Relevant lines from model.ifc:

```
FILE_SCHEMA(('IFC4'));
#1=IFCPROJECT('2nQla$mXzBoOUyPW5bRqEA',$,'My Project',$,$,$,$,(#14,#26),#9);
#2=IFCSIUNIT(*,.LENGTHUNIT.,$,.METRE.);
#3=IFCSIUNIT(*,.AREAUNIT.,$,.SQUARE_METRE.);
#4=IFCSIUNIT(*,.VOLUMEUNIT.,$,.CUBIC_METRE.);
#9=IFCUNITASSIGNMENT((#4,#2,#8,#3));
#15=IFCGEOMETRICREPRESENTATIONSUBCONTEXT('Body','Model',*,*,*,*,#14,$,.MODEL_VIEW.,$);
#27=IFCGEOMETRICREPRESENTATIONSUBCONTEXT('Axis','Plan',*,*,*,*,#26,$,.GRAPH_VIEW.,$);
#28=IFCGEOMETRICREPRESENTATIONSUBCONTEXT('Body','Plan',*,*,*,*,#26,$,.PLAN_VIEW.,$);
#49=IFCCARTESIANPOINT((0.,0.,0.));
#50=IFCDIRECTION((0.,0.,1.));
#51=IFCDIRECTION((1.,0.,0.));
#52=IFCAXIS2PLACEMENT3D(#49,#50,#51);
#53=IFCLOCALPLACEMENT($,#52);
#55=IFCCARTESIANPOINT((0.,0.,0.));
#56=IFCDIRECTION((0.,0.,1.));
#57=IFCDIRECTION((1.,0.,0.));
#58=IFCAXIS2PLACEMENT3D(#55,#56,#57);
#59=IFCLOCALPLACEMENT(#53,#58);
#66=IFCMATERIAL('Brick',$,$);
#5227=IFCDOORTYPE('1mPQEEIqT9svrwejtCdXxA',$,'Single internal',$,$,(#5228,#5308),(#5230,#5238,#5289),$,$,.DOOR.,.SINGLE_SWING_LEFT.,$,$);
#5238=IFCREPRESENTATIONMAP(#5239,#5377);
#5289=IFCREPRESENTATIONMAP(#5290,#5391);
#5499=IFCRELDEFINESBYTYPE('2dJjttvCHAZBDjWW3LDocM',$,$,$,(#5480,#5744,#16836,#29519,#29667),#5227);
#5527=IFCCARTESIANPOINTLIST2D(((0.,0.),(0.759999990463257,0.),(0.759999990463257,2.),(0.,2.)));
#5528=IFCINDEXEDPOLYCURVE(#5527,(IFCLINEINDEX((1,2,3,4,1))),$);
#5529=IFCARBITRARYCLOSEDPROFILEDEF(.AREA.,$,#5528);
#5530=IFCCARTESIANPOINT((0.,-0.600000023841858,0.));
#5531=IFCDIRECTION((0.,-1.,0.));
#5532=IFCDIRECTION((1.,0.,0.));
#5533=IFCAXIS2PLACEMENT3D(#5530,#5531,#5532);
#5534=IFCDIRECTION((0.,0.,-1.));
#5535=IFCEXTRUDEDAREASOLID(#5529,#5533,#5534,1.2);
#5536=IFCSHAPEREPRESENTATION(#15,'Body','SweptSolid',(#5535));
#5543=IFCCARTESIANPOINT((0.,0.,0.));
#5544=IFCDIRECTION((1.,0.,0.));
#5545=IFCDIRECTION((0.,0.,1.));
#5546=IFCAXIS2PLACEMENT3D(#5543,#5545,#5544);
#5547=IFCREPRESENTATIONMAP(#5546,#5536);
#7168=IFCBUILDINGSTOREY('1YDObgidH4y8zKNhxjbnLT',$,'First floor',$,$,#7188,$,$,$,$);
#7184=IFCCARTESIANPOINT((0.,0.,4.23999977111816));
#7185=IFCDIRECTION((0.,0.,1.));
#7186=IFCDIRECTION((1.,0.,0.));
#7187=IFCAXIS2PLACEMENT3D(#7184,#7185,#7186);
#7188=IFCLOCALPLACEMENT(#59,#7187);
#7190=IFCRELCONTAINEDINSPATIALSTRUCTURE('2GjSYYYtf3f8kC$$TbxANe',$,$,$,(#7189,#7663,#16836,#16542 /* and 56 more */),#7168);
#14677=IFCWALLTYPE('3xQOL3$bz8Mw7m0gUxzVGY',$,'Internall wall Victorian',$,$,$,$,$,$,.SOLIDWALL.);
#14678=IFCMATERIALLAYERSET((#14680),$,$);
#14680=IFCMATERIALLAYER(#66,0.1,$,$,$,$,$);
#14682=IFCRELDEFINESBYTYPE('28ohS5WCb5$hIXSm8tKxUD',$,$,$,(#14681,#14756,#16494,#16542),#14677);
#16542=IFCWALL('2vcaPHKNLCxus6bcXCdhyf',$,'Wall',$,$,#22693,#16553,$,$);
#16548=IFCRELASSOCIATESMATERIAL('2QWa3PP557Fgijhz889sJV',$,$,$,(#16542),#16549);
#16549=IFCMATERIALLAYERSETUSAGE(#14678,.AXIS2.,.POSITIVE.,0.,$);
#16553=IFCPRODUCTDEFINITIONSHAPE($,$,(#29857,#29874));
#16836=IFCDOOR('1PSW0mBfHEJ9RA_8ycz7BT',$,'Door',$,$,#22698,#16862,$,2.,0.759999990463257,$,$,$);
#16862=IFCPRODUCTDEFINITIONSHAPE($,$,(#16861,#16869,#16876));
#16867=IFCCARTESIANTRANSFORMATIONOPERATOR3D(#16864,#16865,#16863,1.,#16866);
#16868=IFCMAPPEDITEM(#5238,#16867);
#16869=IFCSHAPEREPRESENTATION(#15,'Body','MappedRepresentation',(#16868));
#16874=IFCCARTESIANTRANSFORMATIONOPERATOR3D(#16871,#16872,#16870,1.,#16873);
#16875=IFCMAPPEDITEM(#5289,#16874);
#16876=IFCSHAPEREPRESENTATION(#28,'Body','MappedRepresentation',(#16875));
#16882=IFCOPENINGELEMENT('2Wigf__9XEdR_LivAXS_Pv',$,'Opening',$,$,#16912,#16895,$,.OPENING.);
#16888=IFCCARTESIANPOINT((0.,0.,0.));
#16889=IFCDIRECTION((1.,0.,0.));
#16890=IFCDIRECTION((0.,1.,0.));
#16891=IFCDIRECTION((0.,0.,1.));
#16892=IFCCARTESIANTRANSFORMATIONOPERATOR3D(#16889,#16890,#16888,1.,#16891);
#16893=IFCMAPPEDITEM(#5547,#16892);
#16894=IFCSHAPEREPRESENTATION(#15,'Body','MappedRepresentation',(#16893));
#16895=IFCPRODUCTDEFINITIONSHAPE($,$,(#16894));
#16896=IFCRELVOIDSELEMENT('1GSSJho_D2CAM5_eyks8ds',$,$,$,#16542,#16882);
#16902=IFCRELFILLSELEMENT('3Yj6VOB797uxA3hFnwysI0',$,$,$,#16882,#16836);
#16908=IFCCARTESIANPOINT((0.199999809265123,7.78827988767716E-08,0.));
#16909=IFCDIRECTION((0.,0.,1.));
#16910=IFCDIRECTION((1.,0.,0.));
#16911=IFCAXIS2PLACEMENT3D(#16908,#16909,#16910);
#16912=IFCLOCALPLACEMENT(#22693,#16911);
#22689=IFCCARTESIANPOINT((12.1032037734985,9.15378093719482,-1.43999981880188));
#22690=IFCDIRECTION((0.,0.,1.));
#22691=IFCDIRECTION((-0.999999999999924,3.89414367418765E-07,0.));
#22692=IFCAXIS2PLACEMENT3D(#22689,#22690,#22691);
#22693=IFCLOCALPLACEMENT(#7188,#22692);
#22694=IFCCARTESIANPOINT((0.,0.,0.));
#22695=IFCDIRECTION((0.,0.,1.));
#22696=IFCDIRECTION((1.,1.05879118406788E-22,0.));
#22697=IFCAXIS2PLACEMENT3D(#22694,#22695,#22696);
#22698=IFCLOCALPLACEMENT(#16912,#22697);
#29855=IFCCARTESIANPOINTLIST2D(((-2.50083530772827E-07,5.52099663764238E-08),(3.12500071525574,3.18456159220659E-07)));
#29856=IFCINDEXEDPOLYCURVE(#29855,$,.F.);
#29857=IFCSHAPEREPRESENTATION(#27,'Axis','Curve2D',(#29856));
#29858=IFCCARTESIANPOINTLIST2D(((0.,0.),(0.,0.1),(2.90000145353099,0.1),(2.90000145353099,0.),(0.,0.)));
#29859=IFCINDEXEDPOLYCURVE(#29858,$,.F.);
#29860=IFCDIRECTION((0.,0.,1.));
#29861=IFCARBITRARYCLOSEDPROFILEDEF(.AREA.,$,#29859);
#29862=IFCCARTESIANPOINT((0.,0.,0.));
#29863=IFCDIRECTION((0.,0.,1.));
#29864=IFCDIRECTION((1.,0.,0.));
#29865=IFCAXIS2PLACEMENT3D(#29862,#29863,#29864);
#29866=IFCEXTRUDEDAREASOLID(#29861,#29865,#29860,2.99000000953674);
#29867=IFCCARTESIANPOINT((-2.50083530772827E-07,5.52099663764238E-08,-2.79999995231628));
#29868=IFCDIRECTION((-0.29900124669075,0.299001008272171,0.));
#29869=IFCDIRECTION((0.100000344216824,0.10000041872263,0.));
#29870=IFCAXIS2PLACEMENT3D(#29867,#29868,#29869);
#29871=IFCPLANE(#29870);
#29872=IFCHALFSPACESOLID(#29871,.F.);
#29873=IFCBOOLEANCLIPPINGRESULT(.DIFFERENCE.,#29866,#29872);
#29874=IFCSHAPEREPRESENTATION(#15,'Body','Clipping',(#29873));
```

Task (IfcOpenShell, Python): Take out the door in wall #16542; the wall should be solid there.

```python
import ifcopenshell
import ifcopenshell.api.feature
import ifcopenshell.api.root
import ifcopenshell.geom
import ifcopenshell.util.shape

model = ifcopenshell.open("model.ifc")
settings = ifcopenshell.geom.settings()


def volume(element):
    """Net volume in cubic metres, openings subtracted."""
    shape = ifcopenshell.geom.create_shape(settings, element)
    return ifcopenshell.util.shape.get_volume(shape.geometry)


door = model.by_guid("1PSW0mBfHEJ9RA_8ycz7BT")
opening = door.FillsVoids[0].RelatingOpeningElement
wall = opening.VoidsElements[0].RelatingBuildingElement
before = volume(wall)

ifcopenshell.api.root.remove_product(model, product=door)
ifcopenshell.api.feature.remove_feature(model, feature=opening)

after = volume(wall)

print(f"wall volume {before:.3f} -> {after:.3f} m3")

model.write("model_v2.ifc")
```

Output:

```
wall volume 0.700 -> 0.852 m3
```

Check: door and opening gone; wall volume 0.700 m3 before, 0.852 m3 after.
